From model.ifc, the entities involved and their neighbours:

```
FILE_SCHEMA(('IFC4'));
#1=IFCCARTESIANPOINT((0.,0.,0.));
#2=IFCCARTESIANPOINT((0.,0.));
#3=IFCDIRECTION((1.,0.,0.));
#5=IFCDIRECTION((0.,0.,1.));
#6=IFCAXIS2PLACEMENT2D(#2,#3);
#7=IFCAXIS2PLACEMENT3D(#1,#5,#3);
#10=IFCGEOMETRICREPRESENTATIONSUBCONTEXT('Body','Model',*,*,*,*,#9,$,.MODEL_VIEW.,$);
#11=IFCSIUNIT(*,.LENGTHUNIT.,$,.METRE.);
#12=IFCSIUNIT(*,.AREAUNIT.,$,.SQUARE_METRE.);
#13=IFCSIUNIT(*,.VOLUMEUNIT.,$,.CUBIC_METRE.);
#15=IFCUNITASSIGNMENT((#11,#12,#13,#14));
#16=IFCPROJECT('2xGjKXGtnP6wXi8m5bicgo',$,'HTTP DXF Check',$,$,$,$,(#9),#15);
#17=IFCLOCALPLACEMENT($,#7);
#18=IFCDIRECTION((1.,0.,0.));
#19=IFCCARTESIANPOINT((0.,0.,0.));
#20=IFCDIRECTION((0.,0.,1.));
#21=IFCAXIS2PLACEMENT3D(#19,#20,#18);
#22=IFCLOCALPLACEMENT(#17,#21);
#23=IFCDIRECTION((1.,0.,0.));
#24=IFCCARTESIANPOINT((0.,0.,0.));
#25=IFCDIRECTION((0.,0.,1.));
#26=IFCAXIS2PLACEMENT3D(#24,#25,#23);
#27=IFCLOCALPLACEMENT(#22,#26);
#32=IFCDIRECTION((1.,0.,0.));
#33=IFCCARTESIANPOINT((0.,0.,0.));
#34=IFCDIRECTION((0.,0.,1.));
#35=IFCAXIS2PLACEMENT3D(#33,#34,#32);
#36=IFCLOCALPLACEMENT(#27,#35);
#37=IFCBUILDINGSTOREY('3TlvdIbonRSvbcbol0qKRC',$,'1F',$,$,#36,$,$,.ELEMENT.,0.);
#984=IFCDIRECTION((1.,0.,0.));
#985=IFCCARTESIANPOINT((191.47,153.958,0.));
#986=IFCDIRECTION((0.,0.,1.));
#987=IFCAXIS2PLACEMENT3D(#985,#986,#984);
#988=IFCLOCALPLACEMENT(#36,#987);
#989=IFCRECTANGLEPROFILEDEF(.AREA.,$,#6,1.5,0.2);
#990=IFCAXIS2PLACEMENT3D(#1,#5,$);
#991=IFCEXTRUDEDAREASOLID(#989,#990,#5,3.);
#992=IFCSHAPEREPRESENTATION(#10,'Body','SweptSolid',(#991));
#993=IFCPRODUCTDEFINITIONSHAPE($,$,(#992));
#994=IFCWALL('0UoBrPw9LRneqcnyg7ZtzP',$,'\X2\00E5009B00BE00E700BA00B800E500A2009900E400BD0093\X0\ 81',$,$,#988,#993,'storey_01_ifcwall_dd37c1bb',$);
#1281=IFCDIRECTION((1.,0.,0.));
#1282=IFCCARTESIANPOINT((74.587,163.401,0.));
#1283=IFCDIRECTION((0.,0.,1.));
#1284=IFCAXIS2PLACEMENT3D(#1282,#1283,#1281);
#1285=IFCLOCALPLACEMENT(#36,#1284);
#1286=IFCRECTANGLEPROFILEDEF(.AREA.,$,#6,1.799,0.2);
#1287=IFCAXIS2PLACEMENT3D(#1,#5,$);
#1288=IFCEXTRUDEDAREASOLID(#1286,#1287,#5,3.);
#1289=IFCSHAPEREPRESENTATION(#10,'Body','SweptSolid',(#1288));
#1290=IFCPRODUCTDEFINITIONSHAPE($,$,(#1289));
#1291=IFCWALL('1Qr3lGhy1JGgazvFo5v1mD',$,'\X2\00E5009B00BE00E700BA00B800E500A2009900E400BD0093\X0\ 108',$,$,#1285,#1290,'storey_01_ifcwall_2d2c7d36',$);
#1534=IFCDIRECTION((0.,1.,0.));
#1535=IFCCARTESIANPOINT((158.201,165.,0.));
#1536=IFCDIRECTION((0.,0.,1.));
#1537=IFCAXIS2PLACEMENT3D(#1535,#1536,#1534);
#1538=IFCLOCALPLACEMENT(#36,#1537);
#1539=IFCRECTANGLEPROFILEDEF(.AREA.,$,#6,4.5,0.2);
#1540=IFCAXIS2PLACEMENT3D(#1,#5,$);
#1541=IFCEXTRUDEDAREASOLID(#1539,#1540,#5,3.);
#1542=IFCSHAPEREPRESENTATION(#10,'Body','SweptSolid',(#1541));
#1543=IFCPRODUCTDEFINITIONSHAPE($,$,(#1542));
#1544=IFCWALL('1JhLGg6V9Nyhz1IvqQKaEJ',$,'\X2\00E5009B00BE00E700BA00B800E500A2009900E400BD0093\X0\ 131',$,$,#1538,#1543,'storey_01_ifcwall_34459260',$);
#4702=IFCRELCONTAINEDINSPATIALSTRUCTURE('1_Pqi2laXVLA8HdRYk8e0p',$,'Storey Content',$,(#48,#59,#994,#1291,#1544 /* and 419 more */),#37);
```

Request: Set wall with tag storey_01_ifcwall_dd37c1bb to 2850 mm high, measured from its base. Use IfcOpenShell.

```python
import ifcopenshell
import ifcopenshell.geom
import ifcopenshell.util.representation
import ifcopenshell.util.shape
import ifcopenshell.util.unit

model = ifcopenshell.open("model.ifc")
unit_scale = ifcopenshell.util.unit.calculate_unit_scale(model)
settings = ifcopenshell.geom.settings()


def volume(element):
    """Net volume in cubic metres, openings subtracted."""
    shape = ifcopenshell.geom.create_shape(settings, element)
    return ifcopenshell.util.shape.get_volume(shape.geometry)


wall = model.by_guid("0UoBrPw9LRneqcnyg7ZtzP")
before = volume(wall)

body = ifcopenshell.util.representation.get_representation(wall, "Model", "Body")
solid = body.Items[0]
old_height = solid.Depth
solid.Depth = 2.85 / unit_scale
after = volume(wall)

print(f"height {old_height:g} -> {solid.Depth:g}, volume {before:.3f} -> {after:.3f} m3")

model.write("model_edited.ifc")
```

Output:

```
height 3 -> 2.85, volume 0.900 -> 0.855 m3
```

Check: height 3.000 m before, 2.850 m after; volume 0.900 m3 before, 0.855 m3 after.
